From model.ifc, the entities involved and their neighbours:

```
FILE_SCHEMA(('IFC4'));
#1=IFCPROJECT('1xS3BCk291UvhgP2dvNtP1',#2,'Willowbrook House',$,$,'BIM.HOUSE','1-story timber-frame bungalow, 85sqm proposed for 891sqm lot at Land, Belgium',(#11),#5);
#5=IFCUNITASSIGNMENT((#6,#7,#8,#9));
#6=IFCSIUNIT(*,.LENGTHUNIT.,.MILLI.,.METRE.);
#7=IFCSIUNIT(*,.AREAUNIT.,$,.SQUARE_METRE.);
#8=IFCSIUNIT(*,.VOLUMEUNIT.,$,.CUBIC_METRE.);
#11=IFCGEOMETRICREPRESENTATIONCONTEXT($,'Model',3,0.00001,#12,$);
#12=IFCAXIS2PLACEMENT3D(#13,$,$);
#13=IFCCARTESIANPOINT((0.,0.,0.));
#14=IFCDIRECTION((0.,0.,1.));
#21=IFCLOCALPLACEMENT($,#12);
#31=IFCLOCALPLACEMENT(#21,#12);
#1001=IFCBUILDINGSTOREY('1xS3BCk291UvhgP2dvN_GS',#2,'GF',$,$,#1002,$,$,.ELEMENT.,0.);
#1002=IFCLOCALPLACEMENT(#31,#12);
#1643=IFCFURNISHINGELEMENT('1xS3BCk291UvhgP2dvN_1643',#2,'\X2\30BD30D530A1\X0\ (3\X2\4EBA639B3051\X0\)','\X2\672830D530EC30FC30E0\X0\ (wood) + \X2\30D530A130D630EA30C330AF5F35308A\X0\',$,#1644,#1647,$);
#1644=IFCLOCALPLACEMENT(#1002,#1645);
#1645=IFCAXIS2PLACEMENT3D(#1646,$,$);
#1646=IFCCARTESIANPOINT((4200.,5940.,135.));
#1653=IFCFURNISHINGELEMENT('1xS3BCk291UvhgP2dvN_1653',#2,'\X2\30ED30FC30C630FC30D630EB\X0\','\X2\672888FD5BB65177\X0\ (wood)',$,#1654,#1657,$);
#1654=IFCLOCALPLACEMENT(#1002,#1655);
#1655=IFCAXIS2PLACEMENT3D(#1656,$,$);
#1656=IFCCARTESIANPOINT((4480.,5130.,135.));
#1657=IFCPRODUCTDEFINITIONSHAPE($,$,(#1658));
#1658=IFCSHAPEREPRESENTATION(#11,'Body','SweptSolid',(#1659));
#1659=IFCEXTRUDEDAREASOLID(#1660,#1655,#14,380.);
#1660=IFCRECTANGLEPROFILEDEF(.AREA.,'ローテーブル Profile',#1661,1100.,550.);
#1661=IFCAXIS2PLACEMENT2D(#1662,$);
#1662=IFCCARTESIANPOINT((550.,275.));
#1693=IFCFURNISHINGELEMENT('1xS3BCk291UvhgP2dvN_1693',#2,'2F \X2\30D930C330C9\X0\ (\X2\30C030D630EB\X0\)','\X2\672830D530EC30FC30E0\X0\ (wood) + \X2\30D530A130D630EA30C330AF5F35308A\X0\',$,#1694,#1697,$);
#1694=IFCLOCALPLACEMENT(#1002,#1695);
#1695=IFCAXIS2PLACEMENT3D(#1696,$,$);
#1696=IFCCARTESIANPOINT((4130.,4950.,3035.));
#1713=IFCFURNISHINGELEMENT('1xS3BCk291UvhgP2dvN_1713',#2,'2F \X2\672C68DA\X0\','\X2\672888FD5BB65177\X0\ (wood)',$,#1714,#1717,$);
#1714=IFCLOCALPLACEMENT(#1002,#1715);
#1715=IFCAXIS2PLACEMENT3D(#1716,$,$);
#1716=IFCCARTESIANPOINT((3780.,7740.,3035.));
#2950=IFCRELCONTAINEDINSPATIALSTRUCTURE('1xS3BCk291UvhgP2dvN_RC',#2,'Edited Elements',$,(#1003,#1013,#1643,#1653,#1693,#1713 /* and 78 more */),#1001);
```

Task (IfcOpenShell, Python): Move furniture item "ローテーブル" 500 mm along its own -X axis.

```python
import ifcopenshell
import ifcopenshell.api.geometry
import ifcopenshell.util.placement
import ifcopenshell.util.unit

model = ifcopenshell.open("model.ifc")
unit_scale = ifcopenshell.util.unit.calculate_unit_scale(model)

item = model.by_id(1653)
matrix = ifcopenshell.util.placement.get_local_placement(item.ObjectPlacement)
matrix[:3, 3] -= matrix[:3, 0] * 0.5 / unit_scale
ifcopenshell.api.geometry.edit_object_placement(model, product=item, matrix=matrix, is_si=False)

print(ifcopenshell.util.placement.get_local_placement(item.ObjectPlacement).round(3) + 0.0)

model.write("model_v2.ifc")
```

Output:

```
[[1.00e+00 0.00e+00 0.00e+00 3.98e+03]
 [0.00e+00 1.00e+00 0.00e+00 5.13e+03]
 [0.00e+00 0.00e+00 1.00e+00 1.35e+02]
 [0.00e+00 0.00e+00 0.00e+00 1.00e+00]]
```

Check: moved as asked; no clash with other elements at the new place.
